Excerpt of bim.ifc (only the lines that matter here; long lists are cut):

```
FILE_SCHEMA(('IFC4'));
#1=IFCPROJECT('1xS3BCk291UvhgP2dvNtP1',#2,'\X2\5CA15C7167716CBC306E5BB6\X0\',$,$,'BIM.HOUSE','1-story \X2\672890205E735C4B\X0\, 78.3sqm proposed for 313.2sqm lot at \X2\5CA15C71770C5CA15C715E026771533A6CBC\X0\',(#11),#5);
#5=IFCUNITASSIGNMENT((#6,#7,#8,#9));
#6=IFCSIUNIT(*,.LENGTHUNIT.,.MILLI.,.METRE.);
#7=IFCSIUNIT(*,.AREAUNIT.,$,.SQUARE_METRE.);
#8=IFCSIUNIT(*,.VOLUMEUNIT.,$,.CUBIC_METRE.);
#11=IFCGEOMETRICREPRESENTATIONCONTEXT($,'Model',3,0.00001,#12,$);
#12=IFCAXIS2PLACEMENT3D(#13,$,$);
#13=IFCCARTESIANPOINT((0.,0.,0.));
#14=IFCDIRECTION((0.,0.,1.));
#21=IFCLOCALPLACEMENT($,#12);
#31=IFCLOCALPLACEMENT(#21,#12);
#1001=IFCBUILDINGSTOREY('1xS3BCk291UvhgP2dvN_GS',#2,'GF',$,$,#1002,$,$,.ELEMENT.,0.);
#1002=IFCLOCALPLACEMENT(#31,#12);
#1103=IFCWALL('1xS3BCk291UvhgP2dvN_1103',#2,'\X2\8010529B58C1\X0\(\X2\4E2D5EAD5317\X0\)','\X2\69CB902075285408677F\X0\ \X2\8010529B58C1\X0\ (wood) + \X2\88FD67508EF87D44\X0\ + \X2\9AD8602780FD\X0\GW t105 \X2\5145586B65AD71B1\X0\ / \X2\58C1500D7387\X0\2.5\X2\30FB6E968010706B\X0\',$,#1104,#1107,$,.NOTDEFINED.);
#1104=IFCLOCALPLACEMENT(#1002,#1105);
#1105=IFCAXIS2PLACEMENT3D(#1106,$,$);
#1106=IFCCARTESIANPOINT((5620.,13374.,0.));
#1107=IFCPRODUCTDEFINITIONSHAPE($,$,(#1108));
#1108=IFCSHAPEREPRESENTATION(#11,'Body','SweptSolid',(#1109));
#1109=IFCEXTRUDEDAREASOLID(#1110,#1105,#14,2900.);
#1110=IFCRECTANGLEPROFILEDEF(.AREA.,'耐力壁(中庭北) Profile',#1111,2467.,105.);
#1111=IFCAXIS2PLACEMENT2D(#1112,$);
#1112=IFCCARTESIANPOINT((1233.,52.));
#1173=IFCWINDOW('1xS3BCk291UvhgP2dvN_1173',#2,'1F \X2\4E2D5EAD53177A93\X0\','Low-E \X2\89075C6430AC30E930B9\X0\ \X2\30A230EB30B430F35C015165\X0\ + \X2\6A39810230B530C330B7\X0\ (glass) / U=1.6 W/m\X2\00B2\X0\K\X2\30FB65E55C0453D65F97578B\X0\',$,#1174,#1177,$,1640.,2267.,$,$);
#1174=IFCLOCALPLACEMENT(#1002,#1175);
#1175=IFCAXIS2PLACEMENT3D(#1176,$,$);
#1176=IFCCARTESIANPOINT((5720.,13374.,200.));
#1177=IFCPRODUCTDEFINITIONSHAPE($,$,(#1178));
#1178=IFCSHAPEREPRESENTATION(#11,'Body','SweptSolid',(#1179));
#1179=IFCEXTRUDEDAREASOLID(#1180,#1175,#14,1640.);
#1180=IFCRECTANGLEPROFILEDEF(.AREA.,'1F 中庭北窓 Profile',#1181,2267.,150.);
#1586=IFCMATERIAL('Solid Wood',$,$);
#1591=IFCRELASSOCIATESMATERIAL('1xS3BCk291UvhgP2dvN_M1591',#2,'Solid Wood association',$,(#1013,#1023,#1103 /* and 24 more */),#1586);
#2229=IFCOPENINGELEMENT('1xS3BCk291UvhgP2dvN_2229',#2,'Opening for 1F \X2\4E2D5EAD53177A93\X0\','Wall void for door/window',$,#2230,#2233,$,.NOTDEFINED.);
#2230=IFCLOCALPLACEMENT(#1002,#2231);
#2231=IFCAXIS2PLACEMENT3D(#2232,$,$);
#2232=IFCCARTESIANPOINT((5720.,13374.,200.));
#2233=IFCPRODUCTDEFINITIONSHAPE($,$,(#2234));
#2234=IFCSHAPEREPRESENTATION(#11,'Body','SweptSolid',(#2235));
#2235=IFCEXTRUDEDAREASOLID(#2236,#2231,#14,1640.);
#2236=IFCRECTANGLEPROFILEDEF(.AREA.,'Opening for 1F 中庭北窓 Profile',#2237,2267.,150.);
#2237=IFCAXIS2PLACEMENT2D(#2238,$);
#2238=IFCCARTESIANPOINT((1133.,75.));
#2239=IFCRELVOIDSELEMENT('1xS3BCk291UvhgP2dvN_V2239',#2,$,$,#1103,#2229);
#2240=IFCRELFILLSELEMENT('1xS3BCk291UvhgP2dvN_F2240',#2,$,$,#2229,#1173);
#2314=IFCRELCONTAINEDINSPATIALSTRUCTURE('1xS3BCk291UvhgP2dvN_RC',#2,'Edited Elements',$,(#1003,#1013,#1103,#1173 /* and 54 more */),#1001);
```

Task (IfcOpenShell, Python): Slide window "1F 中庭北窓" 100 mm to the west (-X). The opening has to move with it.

```python
import ifcopenshell
import ifcopenshell.api.geometry
import ifcopenshell.util.placement
import ifcopenshell.util.unit

model = ifcopenshell.open("bim.ifc")
unit_scale = ifcopenshell.util.unit.calculate_unit_scale(model)

window = model.by_guid("1xS3BCk291UvhgP2dvN_1173")
opening = window.FillsVoids[0].RelatingOpeningElement
wall = opening.VoidsElements[0].RelatingBuildingElement

wall_matrix = ifcopenshell.util.placement.get_local_placement(wall.ObjectPlacement)
shift = wall_matrix[:3, 0] * -0.1 / unit_scale
before = ifcopenshell.util.placement.get_local_placement(window.ObjectPlacement)[:3, 3].copy()

# The window is not placed relative to its opening, so move both.
for product in (opening, window):
    matrix = ifcopenshell.util.placement.get_local_placement(product.ObjectPlacement)
    matrix[:3, 3] += shift
    ifcopenshell.api.geometry.edit_object_placement(model, product=product, matrix=matrix, is_si=False)

after = ifcopenshell.util.placement.get_local_placement(window.ObjectPlacement)[:3, 3]
print("window moved by", (after - before).round(3) + 0.0)

model.write("bim_rev.ifc")
```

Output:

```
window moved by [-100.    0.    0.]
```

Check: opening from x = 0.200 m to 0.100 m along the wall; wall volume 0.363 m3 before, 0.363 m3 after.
